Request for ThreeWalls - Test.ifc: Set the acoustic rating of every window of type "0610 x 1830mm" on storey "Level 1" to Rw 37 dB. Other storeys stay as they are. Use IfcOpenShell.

First a look at what the model holds.

```python
import ifcopenshell
import ifcopenshell.util.element

model = ifcopenshell.open("ThreeWalls - Test.ifc")
print(model.schema)
storey = next(s for s in model.by_type("IfcBuildingStorey") if s.Name == "Level 1")
windows = [e for e in ifcopenshell.util.element.get_decomposition(storey) if e.is_a("IfcWindow")]
seen = {}
for e in windows:
    element_type = ifcopenshell.util.element.get_type(e)
    key = (element_type.Name if element_type != e and element_type else None, ifcopenshell.util.element.get_pset(e, "Pset_WindowCommon", "AcousticRating"))
    seen[key] = seen.get(key, 0) + 1
for (name, value), count in sorted(seen.items(), key=str):
    print(count, "x", name, "|", value)
```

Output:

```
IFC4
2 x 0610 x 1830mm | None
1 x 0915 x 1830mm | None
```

```python
import ifcopenshell
import ifcopenshell.api.pset
import ifcopenshell.util.element

model = ifcopenshell.open("ThreeWalls - Test.ifc")

storey = next(s for s in model.by_type("IfcBuildingStorey") if s.Name == "Level 1")
windows = [e for e in ifcopenshell.util.element.get_decomposition(storey) if e.is_a("IfcWindow")]

count = 0
for e in windows:
    element_type = ifcopenshell.util.element.get_type(e)
    if element_type in (None, e) or element_type.Name != "0610 x 1830mm":
        continue
    # add_pset returns the element's existing set when there is one.
    pset = ifcopenshell.api.pset.add_pset(model, product=e, name="Pset_WindowCommon")
    ifcopenshell.api.pset.edit_pset(model, pset=pset, properties={"AcousticRating": "Rw 37 dB"})
    count += 1

print(count, "windows updated")

model.write("ThreeWalls - Test_edited.ifc")
```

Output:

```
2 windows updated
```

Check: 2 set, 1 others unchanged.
